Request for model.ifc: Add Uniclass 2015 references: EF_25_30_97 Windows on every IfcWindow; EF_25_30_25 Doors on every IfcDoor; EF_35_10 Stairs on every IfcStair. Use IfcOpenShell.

First a look at what the model holds.

```python
import ifcopenshell

model = ifcopenshell.open("model.ifc")
print(model.schema)
print("classifications:", [c.Name for c in model.by_type("IfcClassification")])
for ifc_class in ("IfcDoor", "IfcRoof", "IfcStair", "IfcWall", "IfcWindow"):
    print(ifc_class, len(model.by_type(ifc_class)))
```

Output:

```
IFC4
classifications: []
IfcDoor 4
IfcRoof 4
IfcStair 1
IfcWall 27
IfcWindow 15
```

```python
import ifcopenshell
import ifcopenshell.api.classification

model = ifcopenshell.open("model.ifc")

system = ifcopenshell.api.classification.add_classification(model, classification="Uniclass 2015")

codes = {
    "IfcWindow": ("EF_25_30_97", "Windows"),
    "IfcDoor": ("EF_25_30_25", "Doors"),
    "IfcStair": ("EF_35_10", "Stairs"),
}
for ifc_class, (code, name) in codes.items():
    products = model.by_type(ifc_class)
    ifcopenshell.api.classification.add_reference(
        model, products=products, classification=system, identification=code, name=name
    )
    print(code, len(products))

model.write("model-out.ifc")
```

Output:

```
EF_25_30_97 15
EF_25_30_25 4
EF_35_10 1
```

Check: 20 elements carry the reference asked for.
